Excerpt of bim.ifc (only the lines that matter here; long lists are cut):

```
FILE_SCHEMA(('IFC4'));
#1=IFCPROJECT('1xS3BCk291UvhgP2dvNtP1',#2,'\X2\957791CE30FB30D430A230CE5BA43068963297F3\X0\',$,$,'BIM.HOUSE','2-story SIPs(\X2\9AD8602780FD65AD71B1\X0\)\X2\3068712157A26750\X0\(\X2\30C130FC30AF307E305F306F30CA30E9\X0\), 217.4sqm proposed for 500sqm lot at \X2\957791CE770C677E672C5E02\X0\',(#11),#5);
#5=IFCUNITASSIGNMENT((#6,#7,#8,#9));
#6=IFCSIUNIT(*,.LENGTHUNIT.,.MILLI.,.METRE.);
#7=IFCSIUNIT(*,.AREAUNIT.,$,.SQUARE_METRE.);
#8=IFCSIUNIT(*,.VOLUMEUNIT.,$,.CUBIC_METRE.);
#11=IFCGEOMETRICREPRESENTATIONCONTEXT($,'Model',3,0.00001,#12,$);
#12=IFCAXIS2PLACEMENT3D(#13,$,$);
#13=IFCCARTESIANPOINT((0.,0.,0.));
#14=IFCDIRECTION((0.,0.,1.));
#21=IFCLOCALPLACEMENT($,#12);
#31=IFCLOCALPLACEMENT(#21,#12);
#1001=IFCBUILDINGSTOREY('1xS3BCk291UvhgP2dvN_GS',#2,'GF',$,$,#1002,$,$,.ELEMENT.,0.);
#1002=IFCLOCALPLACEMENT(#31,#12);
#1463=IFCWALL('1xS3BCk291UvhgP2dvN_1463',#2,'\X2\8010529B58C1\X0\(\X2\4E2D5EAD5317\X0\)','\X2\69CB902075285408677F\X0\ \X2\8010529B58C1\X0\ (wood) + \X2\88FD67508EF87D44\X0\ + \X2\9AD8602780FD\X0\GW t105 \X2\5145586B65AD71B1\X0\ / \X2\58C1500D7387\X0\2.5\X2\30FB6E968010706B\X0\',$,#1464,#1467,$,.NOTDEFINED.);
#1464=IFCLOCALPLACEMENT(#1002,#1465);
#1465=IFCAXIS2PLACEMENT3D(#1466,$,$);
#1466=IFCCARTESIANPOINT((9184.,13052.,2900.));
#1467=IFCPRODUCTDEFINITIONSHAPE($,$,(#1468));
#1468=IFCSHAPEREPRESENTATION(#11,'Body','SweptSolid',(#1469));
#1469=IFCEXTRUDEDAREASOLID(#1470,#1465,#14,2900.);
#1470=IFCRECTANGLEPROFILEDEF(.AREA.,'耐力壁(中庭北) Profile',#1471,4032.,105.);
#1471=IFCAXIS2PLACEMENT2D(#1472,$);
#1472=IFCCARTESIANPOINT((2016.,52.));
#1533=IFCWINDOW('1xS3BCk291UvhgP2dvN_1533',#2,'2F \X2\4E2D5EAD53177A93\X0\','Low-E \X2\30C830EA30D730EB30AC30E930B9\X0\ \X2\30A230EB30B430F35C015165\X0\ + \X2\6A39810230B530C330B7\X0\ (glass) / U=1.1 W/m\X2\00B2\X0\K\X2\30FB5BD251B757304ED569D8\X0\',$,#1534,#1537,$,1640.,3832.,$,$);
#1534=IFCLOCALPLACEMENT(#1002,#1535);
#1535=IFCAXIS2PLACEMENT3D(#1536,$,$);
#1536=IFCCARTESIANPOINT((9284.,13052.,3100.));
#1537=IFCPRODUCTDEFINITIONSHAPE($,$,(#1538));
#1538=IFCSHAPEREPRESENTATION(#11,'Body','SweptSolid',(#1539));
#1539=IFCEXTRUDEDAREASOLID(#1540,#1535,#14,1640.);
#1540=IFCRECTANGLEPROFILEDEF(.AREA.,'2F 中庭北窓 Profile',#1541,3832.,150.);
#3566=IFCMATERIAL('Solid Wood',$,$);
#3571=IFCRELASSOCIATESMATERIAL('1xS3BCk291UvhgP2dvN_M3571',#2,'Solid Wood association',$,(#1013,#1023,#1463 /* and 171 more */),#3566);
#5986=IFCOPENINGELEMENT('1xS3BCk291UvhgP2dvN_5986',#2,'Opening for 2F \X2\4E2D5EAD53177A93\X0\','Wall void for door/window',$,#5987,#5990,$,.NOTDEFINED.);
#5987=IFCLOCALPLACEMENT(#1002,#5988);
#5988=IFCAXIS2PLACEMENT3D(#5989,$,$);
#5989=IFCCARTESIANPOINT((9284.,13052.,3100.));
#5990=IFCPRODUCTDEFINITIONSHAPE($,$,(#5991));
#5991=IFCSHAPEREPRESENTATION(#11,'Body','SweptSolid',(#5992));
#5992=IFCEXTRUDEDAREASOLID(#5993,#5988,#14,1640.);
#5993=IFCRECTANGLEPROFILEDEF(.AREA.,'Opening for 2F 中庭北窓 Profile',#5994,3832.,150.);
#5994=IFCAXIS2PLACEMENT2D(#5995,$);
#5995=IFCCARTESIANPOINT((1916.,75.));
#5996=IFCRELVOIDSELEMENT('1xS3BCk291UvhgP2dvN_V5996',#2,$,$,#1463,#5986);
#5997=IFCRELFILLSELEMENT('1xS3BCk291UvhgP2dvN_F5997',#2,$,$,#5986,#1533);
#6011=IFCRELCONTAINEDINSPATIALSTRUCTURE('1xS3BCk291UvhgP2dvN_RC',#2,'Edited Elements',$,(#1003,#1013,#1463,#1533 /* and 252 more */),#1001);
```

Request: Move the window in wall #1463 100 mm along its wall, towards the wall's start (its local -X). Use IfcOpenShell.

```python
import ifcopenshell
import ifcopenshell.api.geometry
import ifcopenshell.util.placement
import ifcopenshell.util.unit

model = ifcopenshell.open("bim.ifc")
unit_scale = ifcopenshell.util.unit.calculate_unit_scale(model)

window = model.by_guid("1xS3BCk291UvhgP2dvN_1533")
opening = window.FillsVoids[0].RelatingOpeningElement
wall = opening.VoidsElements[0].RelatingBuildingElement

wall_matrix = ifcopenshell.util.placement.get_local_placement(wall.ObjectPlacement)
shift = wall_matrix[:3, 0] * -0.1 / unit_scale
before = ifcopenshell.util.placement.get_local_placement(window.ObjectPlacement)[:3, 3].copy()

# The window is not placed relative to its opening, so move both.
for product in (opening, window):
    matrix = ifcopenshell.util.placement.get_local_placement(product.ObjectPlacement)
    matrix[:3, 3] += shift
    ifcopenshell.api.geometry.edit_object_placement(model, product=product, matrix=matrix, is_si=False)

after = ifcopenshell.util.placement.get_local_placement(window.ObjectPlacement)[:3, 3]
print("window moved by", (after - before).round(3) + 0.0)

model.write("bim_edited.ifc")
```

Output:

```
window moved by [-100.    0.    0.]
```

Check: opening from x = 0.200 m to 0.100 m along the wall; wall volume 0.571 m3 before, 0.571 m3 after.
